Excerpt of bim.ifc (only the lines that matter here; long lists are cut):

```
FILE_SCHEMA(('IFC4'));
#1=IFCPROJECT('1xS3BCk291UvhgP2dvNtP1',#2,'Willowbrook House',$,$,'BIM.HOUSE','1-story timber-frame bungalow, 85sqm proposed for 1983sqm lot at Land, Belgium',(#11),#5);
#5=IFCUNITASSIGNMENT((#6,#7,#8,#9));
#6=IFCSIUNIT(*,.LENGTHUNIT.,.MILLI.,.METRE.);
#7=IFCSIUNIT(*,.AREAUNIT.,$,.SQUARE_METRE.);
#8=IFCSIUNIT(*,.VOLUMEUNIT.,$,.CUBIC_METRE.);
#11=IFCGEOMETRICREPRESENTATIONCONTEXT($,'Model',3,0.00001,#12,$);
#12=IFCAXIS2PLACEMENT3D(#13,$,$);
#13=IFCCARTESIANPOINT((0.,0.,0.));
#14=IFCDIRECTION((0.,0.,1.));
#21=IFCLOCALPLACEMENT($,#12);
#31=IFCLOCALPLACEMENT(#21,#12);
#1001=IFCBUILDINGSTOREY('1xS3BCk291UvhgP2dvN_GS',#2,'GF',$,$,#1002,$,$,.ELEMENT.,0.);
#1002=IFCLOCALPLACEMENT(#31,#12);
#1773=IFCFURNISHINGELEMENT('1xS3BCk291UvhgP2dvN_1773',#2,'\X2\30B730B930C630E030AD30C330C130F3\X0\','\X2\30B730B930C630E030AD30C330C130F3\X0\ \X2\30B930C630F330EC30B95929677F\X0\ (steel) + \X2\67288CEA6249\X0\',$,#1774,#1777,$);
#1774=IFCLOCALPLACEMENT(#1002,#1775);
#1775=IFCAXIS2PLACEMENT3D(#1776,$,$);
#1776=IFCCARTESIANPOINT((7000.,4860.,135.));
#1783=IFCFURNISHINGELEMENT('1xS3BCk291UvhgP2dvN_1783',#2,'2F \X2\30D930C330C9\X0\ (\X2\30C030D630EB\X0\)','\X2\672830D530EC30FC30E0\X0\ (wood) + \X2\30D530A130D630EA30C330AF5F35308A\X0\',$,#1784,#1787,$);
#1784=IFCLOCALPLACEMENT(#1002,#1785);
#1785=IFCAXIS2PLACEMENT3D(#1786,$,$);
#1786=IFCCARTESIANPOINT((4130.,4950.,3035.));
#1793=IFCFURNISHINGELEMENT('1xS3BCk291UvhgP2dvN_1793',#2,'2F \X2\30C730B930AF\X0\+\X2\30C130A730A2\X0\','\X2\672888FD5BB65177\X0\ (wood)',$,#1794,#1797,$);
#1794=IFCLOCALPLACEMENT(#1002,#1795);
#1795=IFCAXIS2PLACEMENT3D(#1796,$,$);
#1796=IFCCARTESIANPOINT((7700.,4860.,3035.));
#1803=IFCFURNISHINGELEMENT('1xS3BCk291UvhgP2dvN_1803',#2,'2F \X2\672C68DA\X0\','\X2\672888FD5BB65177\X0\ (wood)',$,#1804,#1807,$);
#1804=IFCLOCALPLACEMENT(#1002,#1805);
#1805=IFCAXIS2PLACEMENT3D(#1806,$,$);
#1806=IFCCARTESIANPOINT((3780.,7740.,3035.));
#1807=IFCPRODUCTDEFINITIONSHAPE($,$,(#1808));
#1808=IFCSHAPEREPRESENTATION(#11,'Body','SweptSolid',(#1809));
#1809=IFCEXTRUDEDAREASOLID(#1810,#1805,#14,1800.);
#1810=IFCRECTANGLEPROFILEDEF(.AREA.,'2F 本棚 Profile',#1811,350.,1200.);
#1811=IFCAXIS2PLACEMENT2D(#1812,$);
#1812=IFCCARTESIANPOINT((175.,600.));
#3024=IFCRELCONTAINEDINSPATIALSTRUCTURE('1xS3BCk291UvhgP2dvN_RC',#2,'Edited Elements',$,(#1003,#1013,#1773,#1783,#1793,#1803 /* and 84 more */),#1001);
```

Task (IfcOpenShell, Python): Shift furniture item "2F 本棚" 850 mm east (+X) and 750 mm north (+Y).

```python
import ifcopenshell
import ifcopenshell.api.geometry
import ifcopenshell.util.placement

model = ifcopenshell.open("bim.ifc")

item = model.by_guid("1xS3BCk291UvhgP2dvN_1803")
matrix = ifcopenshell.util.placement.get_local_placement(item.ObjectPlacement)
matrix[0, 3] += 850.0
matrix[1, 3] += 750.0
ifcopenshell.api.geometry.edit_object_placement(model, product=item, matrix=matrix, is_si=False)

print(ifcopenshell.util.placement.get_local_placement(item.ObjectPlacement).round(3) + 0.0)

model.write("bim_updated.ifc")
```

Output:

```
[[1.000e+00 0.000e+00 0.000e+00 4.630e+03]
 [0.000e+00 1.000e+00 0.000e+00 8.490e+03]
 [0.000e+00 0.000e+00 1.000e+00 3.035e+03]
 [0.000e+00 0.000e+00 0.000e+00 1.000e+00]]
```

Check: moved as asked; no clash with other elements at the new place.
